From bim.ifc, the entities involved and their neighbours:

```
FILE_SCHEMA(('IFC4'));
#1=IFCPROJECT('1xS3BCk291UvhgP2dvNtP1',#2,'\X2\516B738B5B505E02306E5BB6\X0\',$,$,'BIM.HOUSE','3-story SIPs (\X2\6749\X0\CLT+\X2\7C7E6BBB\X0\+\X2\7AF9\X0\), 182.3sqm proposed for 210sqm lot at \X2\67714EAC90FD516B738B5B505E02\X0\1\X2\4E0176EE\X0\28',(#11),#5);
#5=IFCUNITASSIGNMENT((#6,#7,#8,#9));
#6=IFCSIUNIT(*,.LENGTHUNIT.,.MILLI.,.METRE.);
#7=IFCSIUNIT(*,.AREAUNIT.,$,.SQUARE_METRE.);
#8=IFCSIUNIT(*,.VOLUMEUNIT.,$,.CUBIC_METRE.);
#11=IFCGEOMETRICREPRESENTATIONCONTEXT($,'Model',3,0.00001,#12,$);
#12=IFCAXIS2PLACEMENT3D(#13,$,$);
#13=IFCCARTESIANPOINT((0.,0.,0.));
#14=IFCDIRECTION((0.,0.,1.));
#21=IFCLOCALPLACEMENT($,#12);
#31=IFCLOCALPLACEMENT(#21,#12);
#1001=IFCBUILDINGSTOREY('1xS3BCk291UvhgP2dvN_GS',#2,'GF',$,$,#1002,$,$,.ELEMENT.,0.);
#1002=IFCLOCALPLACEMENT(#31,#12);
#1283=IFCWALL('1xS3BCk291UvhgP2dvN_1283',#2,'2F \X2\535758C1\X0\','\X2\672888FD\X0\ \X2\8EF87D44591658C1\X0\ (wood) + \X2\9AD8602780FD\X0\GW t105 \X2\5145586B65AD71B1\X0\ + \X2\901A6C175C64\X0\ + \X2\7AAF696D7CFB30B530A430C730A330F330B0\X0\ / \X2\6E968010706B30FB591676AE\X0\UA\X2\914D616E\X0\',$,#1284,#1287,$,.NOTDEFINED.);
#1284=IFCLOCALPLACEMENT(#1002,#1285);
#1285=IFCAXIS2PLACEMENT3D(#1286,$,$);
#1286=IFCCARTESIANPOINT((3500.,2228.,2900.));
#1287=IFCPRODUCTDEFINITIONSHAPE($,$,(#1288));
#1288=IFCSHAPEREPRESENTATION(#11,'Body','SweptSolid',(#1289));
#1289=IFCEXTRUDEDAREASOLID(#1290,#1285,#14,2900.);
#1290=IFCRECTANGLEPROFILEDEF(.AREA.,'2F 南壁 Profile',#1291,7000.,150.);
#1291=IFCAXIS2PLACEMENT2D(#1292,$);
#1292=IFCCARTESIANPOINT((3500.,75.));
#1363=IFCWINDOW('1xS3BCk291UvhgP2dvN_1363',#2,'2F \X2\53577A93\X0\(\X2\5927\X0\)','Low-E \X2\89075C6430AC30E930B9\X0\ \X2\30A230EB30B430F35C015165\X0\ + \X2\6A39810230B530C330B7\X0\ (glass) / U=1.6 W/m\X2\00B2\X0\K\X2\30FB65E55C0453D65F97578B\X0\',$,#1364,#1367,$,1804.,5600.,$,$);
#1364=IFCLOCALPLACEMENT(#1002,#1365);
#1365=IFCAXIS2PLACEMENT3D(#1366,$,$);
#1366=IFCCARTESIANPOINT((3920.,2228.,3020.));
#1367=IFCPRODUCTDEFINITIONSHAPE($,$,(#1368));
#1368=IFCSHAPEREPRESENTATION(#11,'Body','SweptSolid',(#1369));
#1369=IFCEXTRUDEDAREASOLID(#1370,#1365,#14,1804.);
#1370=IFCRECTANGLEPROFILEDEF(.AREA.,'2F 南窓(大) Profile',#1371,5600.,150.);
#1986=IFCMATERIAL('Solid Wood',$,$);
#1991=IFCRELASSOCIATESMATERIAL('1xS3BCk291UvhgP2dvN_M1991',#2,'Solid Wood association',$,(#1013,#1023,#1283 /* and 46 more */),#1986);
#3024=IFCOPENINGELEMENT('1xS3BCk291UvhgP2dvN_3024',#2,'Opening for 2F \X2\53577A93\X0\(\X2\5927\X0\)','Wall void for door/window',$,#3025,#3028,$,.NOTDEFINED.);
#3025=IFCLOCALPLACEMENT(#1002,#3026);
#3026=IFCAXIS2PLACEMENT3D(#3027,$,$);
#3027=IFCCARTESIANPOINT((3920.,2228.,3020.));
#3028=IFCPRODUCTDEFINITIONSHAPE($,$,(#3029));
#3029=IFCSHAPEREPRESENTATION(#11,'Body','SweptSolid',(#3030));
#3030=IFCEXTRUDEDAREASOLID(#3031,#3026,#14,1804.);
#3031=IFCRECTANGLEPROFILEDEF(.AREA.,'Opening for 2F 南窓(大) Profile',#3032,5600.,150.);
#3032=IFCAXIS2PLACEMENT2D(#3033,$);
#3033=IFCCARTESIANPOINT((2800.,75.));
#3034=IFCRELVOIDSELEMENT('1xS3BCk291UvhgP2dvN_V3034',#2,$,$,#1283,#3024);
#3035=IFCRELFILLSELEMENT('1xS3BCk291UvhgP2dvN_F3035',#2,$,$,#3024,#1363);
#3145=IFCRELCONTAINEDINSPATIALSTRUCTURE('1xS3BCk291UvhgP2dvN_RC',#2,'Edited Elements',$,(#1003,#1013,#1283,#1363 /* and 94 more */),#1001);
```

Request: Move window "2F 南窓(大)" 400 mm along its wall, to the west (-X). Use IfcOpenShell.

```python
import ifcopenshell
import ifcopenshell.api.geometry
import ifcopenshell.util.placement
import ifcopenshell.util.unit

model = ifcopenshell.open("bim.ifc")
unit_scale = ifcopenshell.util.unit.calculate_unit_scale(model)

window = model.by_guid("1xS3BCk291UvhgP2dvN_1363")
opening = window.FillsVoids[0].RelatingOpeningElement
wall = opening.VoidsElements[0].RelatingBuildingElement

wall_matrix = ifcopenshell.util.placement.get_local_placement(wall.ObjectPlacement)
shift = wall_matrix[:3, 0] * -0.4 / unit_scale
before = ifcopenshell.util.placement.get_local_placement(window.ObjectPlacement)[:3, 3].copy()

# The window is not placed relative to its opening, so move both.
for product in (opening, window):
    matrix = ifcopenshell.util.placement.get_local_placement(product.ObjectPlacement)
    matrix[:3, 3] += shift
    ifcopenshell.api.geometry.edit_object_placement(model, product=product, matrix=matrix, is_si=False)

after = ifcopenshell.util.placement.get_local_placement(window.ObjectPlacement)[:3, 3]
print("window moved by", (after - before).round(3) + 0.0)

model.write("bim_edited.ifc")
```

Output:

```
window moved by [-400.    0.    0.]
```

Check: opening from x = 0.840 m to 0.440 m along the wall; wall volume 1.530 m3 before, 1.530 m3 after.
